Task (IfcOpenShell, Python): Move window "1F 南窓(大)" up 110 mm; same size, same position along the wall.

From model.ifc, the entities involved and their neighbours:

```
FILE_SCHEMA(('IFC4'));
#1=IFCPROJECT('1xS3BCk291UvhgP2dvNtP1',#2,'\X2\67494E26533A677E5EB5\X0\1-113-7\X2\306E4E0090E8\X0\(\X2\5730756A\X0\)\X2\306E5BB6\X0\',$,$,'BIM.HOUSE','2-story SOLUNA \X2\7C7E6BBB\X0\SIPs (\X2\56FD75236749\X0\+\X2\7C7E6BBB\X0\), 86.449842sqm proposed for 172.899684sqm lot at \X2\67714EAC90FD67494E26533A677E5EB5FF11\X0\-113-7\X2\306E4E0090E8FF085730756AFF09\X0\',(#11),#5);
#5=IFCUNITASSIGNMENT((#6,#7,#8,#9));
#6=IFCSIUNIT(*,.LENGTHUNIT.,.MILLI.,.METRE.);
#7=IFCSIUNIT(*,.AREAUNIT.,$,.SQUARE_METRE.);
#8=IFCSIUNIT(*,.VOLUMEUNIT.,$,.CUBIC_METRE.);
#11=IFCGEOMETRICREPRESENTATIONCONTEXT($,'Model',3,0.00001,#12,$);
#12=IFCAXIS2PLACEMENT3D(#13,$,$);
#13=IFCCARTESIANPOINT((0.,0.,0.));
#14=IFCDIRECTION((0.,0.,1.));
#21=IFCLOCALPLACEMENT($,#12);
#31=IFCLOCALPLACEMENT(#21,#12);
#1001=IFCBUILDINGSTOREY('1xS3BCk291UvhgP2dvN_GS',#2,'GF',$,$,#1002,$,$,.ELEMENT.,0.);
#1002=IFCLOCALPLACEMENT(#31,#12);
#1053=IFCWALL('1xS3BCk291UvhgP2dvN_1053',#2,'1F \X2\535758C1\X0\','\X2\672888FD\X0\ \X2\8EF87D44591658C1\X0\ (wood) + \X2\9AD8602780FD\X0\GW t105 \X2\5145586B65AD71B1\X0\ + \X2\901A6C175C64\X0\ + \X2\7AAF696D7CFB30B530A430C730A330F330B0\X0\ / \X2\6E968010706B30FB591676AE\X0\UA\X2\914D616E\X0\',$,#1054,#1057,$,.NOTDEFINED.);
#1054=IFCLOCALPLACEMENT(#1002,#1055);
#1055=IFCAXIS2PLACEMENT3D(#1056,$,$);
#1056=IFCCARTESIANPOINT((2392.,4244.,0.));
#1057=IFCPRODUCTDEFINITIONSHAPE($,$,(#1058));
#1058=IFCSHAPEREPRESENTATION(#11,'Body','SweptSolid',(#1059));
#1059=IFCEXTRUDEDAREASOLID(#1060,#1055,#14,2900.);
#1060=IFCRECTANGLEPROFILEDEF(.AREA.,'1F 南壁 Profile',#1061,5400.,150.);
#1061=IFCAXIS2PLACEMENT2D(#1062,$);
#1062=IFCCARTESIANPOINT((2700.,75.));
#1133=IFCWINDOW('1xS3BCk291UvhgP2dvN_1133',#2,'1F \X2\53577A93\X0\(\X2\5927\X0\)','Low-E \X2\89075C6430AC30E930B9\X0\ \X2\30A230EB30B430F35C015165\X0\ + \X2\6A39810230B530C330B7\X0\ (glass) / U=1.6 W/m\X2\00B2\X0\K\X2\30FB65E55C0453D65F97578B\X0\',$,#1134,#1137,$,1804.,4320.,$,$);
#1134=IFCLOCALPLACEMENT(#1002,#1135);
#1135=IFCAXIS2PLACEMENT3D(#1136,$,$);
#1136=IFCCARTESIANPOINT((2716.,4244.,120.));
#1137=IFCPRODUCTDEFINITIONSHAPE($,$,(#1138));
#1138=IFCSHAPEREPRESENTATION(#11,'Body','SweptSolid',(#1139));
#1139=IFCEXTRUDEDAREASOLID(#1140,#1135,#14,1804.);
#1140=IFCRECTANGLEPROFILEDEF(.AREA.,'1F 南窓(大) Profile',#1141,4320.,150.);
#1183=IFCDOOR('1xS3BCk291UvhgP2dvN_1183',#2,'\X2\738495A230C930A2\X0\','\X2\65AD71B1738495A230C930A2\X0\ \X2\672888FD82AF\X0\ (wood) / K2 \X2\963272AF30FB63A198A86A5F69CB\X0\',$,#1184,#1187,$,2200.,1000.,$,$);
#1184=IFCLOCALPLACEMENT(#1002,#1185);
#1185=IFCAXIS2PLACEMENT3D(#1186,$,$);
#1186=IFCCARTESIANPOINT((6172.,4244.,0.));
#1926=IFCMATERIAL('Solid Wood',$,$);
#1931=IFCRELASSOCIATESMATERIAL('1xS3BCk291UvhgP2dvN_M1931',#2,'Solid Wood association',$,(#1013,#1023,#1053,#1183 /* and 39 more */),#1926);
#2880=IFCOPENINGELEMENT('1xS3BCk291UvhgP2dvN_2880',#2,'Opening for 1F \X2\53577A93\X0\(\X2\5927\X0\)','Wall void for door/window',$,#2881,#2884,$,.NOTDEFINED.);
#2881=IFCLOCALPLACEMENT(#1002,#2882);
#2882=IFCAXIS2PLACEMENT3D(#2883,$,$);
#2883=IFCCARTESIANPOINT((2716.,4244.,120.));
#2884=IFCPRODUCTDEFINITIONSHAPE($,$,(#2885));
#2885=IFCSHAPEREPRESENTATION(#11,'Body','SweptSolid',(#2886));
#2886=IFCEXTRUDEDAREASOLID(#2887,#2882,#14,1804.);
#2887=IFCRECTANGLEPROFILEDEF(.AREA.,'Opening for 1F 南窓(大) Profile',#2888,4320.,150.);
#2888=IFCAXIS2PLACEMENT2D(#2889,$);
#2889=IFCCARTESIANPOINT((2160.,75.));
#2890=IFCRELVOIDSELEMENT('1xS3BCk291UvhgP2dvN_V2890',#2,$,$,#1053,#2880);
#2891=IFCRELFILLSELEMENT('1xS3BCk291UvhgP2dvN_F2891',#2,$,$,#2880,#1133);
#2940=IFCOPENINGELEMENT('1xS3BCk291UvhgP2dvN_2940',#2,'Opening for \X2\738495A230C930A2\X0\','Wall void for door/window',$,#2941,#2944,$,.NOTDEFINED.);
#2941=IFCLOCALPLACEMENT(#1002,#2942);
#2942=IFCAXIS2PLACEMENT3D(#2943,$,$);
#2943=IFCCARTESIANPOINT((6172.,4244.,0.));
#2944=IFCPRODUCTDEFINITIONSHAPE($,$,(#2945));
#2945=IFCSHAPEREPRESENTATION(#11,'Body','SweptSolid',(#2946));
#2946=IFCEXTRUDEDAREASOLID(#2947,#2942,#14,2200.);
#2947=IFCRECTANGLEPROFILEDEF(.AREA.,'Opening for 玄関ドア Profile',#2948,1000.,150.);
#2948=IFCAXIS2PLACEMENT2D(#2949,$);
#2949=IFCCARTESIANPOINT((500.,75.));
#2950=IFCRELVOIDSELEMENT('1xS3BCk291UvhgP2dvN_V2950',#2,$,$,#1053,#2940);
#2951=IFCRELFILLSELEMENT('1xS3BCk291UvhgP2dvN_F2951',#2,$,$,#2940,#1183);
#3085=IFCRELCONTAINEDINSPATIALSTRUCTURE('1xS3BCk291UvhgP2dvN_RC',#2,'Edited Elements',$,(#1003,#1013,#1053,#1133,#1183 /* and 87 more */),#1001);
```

```python
import numpy as np
import ifcopenshell
import ifcopenshell.api.geometry
import ifcopenshell.util.placement
import ifcopenshell.util.unit

model = ifcopenshell.open("model.ifc")
unit_scale = ifcopenshell.util.unit.calculate_unit_scale(model)

window = model.by_guid("1xS3BCk291UvhgP2dvN_1133")
opening = window.FillsVoids[0].RelatingOpeningElement
dz = 0.11 / unit_scale

shift = np.array([0.0, 0.0, dz])
# The window is not placed relative to its opening, so move both.
for product in (opening, window):
    matrix = ifcopenshell.util.placement.get_local_placement(product.ObjectPlacement)
    matrix[:3, 3] += shift
    ifcopenshell.api.geometry.edit_object_placement(model, product=product, matrix=matrix, is_si=False)

print(f"moved by {dz * unit_scale:+.3f} m")

model.write("model_edited.ifc")
```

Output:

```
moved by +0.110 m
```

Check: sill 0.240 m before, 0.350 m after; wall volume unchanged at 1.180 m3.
